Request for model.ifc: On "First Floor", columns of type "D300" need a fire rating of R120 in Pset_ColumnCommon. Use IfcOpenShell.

First a look at what the model holds.

```python
import ifcopenshell
import ifcopenshell.util.element

model = ifcopenshell.open("model.ifc")
print(model.schema)
storey = next(s for s in model.by_type("IfcBuildingStorey") if s.Name == "First Floor")
columns = [e for e in ifcopenshell.util.element.get_decomposition(storey) if e.is_a("IfcColumn")]
seen = {}
for e in columns:
    element_type = ifcopenshell.util.element.get_type(e)
    key = (element_type.Name if element_type != e and element_type else None, ifcopenshell.util.element.get_pset(e, "Pset_ColumnCommon", "FireRating"))
    seen[key] = seen.get(key, 0) + 1
for (name, value), count in sorted(seen.items(), key=str):
    print(count, "x", name, "|", value)
```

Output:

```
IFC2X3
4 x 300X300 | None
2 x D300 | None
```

```python
import ifcopenshell
import ifcopenshell.api.pset
import ifcopenshell.util.element

model = ifcopenshell.open("model.ifc")

storey = next(s for s in model.by_type("IfcBuildingStorey") if s.Name == "First Floor")
columns = [e for e in ifcopenshell.util.element.get_decomposition(storey) if e.is_a("IfcColumn")]

count = 0
for e in columns:
    element_type = ifcopenshell.util.element.get_type(e)
    if element_type in (None, e) or element_type.Name != "D300":
        continue
    # add_pset returns the element's existing set when there is one.
    pset = ifcopenshell.api.pset.add_pset(model, product=e, name="Pset_ColumnCommon")
    ifcopenshell.api.pset.edit_pset(model, pset=pset, properties={"FireRating": "R120"})
    count += 1

print(count, "columns updated")

model.write("model-out.ifc")
```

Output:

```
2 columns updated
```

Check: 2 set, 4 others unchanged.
